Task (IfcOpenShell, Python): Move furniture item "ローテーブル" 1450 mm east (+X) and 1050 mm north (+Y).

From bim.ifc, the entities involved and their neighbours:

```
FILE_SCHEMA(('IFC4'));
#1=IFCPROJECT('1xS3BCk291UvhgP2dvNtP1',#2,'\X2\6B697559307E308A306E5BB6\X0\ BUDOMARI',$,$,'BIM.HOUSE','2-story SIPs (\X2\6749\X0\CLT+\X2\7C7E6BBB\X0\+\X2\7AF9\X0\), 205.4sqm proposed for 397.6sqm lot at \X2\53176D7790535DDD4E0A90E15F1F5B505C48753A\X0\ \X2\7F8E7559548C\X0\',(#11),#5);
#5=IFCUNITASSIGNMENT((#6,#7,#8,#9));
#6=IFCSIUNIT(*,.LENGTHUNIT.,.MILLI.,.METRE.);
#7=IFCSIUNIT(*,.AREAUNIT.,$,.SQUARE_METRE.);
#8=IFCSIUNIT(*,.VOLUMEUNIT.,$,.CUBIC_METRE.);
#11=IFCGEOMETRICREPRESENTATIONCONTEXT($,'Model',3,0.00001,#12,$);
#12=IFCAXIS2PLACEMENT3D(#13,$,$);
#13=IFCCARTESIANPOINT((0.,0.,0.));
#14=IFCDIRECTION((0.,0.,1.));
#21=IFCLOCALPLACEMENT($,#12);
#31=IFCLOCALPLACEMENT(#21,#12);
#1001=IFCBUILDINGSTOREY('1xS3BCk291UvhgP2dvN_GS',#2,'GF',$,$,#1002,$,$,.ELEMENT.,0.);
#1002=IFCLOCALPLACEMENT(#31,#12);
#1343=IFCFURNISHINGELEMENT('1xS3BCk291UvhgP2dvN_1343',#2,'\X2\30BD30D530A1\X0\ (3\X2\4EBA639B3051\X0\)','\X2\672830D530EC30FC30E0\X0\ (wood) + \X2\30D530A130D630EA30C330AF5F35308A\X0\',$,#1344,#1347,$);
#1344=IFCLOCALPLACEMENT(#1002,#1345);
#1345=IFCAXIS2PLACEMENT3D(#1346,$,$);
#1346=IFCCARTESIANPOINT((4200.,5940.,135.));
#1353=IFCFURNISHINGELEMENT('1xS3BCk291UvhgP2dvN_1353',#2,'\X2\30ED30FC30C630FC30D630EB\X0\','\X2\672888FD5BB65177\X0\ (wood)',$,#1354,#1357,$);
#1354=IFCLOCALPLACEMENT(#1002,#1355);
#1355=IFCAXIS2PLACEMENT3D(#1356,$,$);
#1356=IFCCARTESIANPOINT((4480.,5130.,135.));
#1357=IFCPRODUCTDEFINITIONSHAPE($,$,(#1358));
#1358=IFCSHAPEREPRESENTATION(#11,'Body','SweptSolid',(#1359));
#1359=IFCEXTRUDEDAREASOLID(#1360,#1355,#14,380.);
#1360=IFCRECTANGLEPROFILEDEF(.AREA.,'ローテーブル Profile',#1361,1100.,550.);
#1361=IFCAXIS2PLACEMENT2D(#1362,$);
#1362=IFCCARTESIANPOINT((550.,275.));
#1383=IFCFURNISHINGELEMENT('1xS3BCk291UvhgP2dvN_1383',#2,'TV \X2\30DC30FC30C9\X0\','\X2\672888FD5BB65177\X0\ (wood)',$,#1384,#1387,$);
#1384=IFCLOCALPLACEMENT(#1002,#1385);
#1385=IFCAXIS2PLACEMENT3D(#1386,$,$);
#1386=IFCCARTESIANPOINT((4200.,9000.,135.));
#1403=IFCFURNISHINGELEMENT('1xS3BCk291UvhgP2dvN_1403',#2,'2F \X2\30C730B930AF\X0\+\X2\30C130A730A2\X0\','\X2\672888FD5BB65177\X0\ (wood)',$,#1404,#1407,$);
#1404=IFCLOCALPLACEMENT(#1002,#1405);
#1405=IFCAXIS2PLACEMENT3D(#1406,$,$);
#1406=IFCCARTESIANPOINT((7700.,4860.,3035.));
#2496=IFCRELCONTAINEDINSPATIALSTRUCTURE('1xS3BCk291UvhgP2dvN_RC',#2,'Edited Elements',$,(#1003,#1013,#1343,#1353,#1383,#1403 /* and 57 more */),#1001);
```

```python
import ifcopenshell
import ifcopenshell.api.geometry
import ifcopenshell.util.placement
import ifcopenshell.util.unit

model = ifcopenshell.open("bim.ifc")
unit_scale = ifcopenshell.util.unit.calculate_unit_scale(model)

item = model.by_guid("1xS3BCk291UvhgP2dvN_1353")
matrix = ifcopenshell.util.placement.get_local_placement(item.ObjectPlacement)
matrix[0, 3] += 1.45 / unit_scale
matrix[1, 3] += 1.05 / unit_scale
ifcopenshell.api.geometry.edit_object_placement(model, product=item, matrix=matrix, is_si=False)

print(ifcopenshell.util.placement.get_local_placement(item.ObjectPlacement).round(3) + 0.0)

model.write("bim_v2.ifc")
```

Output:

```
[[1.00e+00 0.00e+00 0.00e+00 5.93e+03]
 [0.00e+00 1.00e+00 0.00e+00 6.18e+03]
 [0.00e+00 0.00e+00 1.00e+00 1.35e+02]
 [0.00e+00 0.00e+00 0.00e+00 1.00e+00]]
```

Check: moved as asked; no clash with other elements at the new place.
